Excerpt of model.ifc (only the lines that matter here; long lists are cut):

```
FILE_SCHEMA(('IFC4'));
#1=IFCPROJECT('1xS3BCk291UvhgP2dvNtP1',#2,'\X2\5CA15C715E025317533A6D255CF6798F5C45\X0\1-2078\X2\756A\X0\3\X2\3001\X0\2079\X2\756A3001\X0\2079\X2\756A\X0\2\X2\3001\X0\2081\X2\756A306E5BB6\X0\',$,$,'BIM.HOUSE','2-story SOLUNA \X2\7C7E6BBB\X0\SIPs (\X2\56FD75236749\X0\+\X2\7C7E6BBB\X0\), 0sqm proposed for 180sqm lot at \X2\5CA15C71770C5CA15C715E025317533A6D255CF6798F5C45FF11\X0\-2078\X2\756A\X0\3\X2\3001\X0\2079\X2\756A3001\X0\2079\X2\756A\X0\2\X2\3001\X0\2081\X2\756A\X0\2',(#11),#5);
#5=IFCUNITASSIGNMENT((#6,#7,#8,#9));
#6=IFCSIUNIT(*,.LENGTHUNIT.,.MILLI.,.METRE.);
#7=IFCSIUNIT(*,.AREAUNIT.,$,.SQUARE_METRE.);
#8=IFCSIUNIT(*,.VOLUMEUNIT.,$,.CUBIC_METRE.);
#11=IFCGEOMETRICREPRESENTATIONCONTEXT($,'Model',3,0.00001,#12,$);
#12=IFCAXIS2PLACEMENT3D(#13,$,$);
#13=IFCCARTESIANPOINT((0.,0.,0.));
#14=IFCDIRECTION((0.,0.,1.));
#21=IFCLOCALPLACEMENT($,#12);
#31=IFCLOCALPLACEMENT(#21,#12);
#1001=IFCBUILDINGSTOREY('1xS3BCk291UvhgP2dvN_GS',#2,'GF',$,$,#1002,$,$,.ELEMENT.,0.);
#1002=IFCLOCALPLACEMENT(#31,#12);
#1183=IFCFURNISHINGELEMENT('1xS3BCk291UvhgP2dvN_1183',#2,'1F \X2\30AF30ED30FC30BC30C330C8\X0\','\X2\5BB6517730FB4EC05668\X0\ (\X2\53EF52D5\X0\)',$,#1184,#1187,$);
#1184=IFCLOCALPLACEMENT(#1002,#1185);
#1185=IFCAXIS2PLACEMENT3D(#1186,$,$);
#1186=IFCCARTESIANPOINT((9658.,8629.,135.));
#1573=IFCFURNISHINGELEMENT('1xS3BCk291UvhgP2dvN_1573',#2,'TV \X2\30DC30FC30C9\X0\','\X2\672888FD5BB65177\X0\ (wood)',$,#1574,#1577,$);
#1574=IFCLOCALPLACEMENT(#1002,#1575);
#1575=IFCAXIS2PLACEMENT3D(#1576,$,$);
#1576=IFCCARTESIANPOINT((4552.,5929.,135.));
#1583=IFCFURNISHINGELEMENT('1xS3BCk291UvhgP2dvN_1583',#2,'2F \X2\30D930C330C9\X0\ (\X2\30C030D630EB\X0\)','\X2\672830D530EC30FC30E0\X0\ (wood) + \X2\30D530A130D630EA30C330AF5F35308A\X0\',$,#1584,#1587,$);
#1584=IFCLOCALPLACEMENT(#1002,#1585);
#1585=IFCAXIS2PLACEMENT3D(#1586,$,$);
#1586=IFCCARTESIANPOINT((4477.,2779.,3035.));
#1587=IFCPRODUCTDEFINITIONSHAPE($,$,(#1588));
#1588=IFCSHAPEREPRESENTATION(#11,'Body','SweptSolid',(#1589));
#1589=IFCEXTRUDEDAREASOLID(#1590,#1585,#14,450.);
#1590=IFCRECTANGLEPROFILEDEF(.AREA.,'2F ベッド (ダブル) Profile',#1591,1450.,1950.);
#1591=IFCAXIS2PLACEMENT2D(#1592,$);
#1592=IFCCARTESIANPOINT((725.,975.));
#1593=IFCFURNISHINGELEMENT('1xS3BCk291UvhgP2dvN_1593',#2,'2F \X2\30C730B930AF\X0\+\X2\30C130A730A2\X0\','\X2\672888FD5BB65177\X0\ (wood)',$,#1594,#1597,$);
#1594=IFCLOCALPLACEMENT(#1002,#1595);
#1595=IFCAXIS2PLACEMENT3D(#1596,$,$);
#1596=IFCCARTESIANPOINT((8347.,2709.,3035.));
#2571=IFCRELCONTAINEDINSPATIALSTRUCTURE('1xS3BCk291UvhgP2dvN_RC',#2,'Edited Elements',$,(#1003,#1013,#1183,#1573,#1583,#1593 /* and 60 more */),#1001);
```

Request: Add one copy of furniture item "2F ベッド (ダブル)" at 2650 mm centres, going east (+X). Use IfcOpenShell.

```python
import numpy as np
import ifcopenshell
import ifcopenshell.api.geometry
import ifcopenshell.api.root
import ifcopenshell.util.element
import ifcopenshell.util.placement
import ifcopenshell.util.unit

model = ifcopenshell.open("model.ifc")
unit_scale = ifcopenshell.util.unit.calculate_unit_scale(model)


def reuse_history(source, copy):
    """copy_class also copies each property set's owner history, people and application; keep the originals."""
    for rel in copy.IsDefinedBy:
        if rel.is_a("IfcRelDefinesByProperties") and (history := rel.RelatingPropertyDefinition.OwnerHistory):
            rel.RelatingPropertyDefinition.OwnerHistory = source.OwnerHistory
            ifcopenshell.util.element.remove_deep2(model, history)


source = model.by_guid("1xS3BCk291UvhgP2dvN_1583")
base = ifcopenshell.util.placement.get_local_placement(source.ObjectPlacement)
step = np.array([1.0, 0.0, 0.0]) * 2.65 / unit_scale

for i in range(1, 2):
    copy = ifcopenshell.api.root.copy_class(model, product=source)
    copy.Representation = ifcopenshell.util.element.copy_deep(
        model, source.Representation, exclude=["IfcGeometricRepresentationContext", "IfcRepresentationMap"]
    )
    reuse_history(source, copy)
    matrix = base.copy()
    matrix[:3, 3] += i * step
    print("added at", matrix[:3, 3].round(3) + 0.0)
    ifcopenshell.api.geometry.edit_object_placement(model, product=copy, matrix=matrix, is_si=False)

model.write("model_edited.ifc")
```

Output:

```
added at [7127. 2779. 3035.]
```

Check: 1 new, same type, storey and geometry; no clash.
